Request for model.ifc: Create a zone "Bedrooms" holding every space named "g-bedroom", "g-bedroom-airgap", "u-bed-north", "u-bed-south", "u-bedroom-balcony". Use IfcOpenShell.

First a look at what the model holds.

```python
import ifcopenshell

model = ifcopenshell.open("model.ifc")
print(model.schema)
seen = {}
for space in model.by_type("IfcSpace"):
    seen[space.LongName] = seen.get(space.LongName, 0) + 1
for name, count in sorted(seen.items(), key=str):
    print(count, "x", name)
print("zones:", [z.Name for z in model.by_type("IfcZone")][:20])
```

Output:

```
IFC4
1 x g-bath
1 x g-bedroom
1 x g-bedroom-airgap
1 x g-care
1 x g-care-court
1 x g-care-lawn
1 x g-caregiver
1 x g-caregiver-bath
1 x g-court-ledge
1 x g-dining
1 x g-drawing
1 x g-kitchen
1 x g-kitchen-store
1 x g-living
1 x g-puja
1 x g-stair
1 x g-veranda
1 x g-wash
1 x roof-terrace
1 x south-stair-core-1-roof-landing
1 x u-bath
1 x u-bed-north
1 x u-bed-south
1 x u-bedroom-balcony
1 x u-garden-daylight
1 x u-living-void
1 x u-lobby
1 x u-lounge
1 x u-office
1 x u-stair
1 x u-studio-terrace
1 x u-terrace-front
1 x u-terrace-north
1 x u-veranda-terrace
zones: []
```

```python
import ifcopenshell
import ifcopenshell.api.group
import ifcopenshell.api.root

model = ifcopenshell.open("model.ifc")

names = {"g-bedroom", "g-bedroom-airgap", "u-bed-north", "u-bed-south", "u-bedroom-balcony"}
spaces = [s for s in model.by_type("IfcSpace") if s.LongName in names]

zone = ifcopenshell.api.root.create_entity(model, ifc_class="IfcZone", name="Bedrooms")
ifcopenshell.api.group.assign_group(model, products=spaces, group=zone)
print(len(spaces), "spaces in", zone.Name)

model.write("model_v2.ifc")
```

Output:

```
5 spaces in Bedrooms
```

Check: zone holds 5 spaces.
